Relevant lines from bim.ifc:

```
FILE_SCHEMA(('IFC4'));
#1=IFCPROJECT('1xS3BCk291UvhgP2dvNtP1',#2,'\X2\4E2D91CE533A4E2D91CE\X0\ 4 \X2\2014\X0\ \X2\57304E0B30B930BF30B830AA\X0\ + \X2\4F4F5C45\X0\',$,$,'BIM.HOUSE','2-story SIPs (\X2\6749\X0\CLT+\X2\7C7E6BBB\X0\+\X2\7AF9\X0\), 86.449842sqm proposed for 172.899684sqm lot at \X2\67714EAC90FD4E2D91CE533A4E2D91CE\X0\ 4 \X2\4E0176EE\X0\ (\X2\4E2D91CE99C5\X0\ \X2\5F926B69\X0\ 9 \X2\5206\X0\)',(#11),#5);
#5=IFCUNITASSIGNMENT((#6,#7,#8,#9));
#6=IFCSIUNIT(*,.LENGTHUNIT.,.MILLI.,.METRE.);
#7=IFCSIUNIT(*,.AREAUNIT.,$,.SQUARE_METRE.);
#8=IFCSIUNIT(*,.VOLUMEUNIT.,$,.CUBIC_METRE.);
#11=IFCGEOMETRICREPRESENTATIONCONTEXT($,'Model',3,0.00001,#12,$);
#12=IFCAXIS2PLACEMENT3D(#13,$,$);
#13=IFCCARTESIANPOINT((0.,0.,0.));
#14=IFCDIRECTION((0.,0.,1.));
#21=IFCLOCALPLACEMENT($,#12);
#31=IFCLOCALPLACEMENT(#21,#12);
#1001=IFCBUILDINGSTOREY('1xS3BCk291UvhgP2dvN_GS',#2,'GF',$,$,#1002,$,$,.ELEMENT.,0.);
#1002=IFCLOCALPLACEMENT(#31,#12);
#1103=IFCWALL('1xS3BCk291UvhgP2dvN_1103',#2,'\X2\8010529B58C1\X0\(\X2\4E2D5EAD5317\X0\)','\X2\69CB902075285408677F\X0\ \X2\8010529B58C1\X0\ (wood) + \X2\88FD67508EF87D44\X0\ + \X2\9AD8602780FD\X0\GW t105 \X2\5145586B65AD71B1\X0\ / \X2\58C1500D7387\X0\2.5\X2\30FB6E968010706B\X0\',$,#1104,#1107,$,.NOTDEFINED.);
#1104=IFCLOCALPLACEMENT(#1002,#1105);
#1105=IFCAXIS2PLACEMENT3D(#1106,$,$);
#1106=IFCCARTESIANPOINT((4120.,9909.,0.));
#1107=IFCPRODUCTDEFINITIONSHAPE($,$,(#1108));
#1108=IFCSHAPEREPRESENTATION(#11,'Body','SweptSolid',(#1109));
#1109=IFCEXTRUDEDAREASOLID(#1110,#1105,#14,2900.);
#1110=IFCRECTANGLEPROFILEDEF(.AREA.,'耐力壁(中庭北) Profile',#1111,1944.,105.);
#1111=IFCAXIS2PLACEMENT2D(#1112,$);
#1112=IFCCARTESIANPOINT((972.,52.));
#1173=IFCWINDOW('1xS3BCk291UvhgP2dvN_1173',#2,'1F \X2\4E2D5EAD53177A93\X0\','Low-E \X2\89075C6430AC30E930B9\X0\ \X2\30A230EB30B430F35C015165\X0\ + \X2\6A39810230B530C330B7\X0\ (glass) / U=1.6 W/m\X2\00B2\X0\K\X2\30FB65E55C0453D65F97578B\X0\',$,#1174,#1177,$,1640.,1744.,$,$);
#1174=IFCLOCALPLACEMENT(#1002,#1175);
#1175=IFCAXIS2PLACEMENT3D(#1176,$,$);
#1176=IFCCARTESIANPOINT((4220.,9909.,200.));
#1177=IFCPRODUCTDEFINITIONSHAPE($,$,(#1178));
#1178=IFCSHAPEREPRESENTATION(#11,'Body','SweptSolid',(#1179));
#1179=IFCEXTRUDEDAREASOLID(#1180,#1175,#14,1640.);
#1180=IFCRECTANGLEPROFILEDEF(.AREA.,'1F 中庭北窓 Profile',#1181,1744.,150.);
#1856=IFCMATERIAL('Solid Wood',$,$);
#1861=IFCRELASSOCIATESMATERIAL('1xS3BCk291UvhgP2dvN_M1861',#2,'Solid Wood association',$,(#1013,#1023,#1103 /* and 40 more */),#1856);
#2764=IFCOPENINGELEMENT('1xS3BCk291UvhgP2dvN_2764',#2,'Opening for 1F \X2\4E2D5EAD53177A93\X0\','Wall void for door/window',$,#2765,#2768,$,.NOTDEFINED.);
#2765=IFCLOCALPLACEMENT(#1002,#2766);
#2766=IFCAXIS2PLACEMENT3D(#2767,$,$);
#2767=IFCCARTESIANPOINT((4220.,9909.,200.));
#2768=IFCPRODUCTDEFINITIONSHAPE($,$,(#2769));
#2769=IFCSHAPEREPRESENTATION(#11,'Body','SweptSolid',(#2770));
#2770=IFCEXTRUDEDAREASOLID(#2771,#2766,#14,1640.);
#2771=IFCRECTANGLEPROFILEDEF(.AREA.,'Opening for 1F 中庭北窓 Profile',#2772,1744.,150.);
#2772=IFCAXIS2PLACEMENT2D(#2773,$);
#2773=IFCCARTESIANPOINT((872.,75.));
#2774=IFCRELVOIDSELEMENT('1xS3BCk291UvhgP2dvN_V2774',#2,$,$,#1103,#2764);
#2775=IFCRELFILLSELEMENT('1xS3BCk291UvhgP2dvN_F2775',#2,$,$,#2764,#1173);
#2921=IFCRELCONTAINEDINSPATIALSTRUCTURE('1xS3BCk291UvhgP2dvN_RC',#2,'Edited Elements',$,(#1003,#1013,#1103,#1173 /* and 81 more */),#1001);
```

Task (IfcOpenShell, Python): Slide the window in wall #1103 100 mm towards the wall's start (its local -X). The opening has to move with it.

```python
import ifcopenshell
import ifcopenshell.api.geometry
import ifcopenshell.util.placement
import ifcopenshell.util.unit

model = ifcopenshell.open("bim.ifc")
unit_scale = ifcopenshell.util.unit.calculate_unit_scale(model)

window = model.by_id(1173)
opening = window.FillsVoids[0].RelatingOpeningElement
wall = opening.VoidsElements[0].RelatingBuildingElement

wall_matrix = ifcopenshell.util.placement.get_local_placement(wall.ObjectPlacement)
shift = wall_matrix[:3, 0] * -0.1 / unit_scale
before = ifcopenshell.util.placement.get_local_placement(window.ObjectPlacement)[:3, 3].copy()

# The window is not placed relative to its opening, so move both.
for product in (opening, window):
    matrix = ifcopenshell.util.placement.get_local_placement(product.ObjectPlacement)
    matrix[:3, 3] += shift
    ifcopenshell.api.geometry.edit_object_placement(model, product=product, matrix=matrix, is_si=False)

after = ifcopenshell.util.placement.get_local_placement(window.ObjectPlacement)[:3, 3]
print("window moved by", (after - before).round(3) + 0.0)

model.write("bim_rev.ifc")
```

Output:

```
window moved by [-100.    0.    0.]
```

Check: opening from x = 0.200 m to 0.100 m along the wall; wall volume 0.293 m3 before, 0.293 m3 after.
